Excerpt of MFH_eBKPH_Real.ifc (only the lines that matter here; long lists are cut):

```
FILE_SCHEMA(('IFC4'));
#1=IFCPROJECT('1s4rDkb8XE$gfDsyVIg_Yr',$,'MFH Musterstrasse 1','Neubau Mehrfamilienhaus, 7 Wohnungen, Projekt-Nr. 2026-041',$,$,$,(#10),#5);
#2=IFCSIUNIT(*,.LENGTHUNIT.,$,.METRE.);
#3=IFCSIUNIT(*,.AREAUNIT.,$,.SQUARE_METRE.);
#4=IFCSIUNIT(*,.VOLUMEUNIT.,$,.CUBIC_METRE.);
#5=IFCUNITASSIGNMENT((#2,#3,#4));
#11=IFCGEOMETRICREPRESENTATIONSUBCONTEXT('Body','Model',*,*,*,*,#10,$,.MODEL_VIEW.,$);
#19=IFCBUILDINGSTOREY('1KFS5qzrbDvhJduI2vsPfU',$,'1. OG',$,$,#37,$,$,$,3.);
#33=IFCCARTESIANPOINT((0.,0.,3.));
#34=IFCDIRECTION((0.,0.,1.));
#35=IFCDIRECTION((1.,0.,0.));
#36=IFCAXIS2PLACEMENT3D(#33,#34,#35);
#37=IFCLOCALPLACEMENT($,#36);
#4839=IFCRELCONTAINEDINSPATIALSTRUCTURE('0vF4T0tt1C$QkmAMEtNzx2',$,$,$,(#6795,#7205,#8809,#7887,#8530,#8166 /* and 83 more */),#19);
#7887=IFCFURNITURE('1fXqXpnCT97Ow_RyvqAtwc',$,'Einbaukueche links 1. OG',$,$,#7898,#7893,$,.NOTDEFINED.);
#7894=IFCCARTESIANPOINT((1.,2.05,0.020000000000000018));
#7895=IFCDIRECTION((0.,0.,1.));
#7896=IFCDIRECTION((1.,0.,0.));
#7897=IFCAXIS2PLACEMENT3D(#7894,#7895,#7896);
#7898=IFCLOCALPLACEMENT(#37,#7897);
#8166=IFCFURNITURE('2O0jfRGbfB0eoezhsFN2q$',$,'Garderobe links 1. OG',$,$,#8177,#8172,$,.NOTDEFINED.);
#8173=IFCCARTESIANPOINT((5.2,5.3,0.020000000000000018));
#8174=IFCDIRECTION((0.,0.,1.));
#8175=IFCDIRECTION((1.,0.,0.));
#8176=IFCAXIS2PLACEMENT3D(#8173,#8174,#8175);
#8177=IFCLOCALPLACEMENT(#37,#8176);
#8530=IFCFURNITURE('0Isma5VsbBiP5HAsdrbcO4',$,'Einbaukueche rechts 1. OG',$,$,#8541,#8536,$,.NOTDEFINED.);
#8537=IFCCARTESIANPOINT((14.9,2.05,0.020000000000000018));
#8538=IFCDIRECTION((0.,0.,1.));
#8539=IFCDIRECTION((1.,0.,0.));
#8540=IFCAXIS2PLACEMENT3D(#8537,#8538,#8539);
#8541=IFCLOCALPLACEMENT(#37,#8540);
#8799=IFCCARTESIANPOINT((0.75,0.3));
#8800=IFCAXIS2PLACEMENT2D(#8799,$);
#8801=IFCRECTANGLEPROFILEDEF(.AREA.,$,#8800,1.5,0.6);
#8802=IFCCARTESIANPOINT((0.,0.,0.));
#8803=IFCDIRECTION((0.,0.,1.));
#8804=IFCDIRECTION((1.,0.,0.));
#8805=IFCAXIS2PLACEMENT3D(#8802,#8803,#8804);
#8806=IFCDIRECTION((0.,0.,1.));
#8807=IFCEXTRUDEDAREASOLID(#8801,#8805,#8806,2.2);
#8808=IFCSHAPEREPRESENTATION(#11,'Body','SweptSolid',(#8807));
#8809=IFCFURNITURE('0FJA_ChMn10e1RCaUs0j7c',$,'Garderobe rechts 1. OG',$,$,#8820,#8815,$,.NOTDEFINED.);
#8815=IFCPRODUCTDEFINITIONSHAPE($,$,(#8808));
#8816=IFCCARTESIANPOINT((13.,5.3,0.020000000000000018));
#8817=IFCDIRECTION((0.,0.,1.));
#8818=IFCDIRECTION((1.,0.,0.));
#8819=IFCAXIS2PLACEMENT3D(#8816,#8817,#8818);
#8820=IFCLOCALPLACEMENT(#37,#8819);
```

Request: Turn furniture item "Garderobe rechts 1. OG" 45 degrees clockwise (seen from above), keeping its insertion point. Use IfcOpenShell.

```python
import ifcopenshell
import ifcopenshell.api.geometry
import ifcopenshell.util.placement

model = ifcopenshell.open("MFH_eBKPH_Real.ifc")

item = model.by_guid("0FJA_ChMn10e1RCaUs0j7c")
matrix = ifcopenshell.util.placement.get_local_placement(item.ObjectPlacement)
matrix = matrix @ ifcopenshell.util.placement.rotation(-45, "Z")
ifcopenshell.api.geometry.edit_object_placement(model, product=item, matrix=matrix, is_si=False)

print(ifcopenshell.util.placement.get_local_placement(item.ObjectPlacement).round(3) + 0.0)

model.write("MFH_eBKPH_Real_updated.ifc")
```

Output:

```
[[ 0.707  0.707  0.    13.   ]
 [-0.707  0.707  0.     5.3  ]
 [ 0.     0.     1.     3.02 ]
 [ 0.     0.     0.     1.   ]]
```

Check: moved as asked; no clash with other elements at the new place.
